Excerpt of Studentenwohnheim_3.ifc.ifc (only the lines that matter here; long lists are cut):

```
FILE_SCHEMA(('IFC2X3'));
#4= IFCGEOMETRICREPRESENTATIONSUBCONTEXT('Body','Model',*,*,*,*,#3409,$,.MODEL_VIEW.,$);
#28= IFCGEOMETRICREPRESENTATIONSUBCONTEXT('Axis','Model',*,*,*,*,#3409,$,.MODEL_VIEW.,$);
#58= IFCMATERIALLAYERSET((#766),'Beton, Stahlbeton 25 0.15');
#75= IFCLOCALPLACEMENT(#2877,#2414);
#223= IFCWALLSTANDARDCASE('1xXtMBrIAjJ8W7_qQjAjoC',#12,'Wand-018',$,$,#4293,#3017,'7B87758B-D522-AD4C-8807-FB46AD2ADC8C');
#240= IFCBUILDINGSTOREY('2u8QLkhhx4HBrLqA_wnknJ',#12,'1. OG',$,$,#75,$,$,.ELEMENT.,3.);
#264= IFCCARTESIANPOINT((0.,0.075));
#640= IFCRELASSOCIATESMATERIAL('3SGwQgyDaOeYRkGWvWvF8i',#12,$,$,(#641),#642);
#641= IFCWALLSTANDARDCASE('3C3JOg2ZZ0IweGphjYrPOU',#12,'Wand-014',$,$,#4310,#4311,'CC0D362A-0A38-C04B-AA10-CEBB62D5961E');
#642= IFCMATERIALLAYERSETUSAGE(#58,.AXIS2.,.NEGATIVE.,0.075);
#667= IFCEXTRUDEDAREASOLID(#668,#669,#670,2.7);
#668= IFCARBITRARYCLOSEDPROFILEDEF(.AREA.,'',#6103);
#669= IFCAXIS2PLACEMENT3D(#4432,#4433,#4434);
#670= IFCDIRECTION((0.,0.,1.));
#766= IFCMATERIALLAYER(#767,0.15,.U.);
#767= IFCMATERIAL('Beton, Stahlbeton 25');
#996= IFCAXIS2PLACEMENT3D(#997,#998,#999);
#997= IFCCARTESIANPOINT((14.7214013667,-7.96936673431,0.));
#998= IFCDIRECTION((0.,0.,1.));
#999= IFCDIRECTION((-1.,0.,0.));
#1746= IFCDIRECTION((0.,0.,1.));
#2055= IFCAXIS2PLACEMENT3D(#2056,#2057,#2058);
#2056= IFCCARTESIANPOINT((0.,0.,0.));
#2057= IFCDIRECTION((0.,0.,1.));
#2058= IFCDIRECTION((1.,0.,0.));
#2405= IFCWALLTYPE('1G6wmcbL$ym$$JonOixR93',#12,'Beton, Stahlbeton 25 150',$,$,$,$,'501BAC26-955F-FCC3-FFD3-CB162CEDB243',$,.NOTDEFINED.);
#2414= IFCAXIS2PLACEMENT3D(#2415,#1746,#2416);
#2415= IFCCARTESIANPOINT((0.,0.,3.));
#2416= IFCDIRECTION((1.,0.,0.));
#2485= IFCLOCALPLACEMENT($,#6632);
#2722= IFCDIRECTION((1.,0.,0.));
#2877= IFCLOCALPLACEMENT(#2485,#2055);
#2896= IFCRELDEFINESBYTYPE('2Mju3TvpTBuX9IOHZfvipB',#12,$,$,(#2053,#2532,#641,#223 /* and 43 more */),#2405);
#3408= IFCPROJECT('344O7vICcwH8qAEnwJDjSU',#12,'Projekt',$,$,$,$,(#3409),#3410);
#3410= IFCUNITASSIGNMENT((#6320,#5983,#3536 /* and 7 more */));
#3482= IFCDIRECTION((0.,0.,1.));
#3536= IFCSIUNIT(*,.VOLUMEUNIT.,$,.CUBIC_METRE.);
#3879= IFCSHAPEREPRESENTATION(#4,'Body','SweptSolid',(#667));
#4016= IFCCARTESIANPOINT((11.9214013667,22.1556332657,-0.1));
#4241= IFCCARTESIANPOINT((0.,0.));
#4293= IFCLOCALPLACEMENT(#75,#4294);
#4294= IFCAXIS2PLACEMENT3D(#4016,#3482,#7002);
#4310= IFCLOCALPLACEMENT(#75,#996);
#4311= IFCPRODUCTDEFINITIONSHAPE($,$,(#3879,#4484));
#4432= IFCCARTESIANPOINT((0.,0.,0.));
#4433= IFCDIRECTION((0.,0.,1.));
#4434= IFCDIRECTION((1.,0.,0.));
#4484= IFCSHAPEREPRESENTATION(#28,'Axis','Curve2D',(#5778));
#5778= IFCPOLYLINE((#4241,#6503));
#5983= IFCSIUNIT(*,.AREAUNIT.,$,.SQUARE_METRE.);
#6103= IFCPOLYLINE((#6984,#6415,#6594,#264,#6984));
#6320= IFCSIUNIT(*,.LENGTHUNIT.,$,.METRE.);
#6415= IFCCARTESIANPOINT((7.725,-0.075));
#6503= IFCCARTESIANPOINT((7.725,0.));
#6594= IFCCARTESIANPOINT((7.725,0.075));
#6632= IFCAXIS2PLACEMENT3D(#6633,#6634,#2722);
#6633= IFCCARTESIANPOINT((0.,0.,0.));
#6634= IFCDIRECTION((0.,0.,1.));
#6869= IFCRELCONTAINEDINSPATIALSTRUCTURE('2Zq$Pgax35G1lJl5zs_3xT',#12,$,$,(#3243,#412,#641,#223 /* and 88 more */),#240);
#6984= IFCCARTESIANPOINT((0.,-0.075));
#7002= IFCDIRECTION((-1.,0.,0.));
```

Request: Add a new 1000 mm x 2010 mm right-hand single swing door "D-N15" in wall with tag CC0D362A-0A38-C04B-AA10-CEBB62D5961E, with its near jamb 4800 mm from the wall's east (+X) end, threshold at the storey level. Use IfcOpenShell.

```python
import numpy as np
import ifcopenshell
import ifcopenshell.api.feature
import ifcopenshell.api.geometry
import ifcopenshell.api.root
import ifcopenshell.api.spatial
import ifcopenshell.api.type
import ifcopenshell.geom
import ifcopenshell.util.element
import ifcopenshell.util.placement
import ifcopenshell.util.representation
import ifcopenshell.util.shape
import ifcopenshell.util.unit

model = ifcopenshell.open("Studentenwohnheim_3.ifc.ifc")
unit_scale = ifcopenshell.util.unit.calculate_unit_scale(model)
settings = ifcopenshell.geom.settings()


def volume(element):
    """Net volume in cubic metres, openings subtracted."""
    shape = ifcopenshell.geom.create_shape(settings, element)
    return ifcopenshell.util.shape.get_volume(shape.geometry)


wall = model.by_id(641)
storey = ifcopenshell.util.element.get_container(wall, ifc_class="IfcBuildingStorey")
context = ifcopenshell.util.representation.get_context(model, "Model", "Body", "MODEL_VIEW")
before = volume(wall)

width, height, from_end, sill = 1, 2.01, 4.8, 0.0  # metres

# The wall runs along its own X axis, and the end named is its -X end.
wall_shape = ifcopenshell.geom.create_shape(settings, wall)
x, y, z = ifcopenshell.util.shape.get_vertices(wall_shape.geometry).T
start = x.min() + from_end
face, thickness = float(y.min()), float(y.max() - y.min())
wall_matrix = ifcopenshell.util.placement.get_local_placement(wall.ObjectPlacement)
level = ifcopenshell.util.placement.get_local_placement(storey.ObjectPlacement)[2, 3]


def in_wall(x, y):
    """Placement at x, y metres in the wall's axes, at sill height."""
    matrix = wall_matrix.copy()
    matrix[:, 3] = wall_matrix @ np.array([x / unit_scale, y / unit_scale, 0.0, 1.0])
    matrix[2, 3] = level + sill / unit_scale
    return matrix


# Opening: a box that overshoots both wall faces by 50 mm.
opening = ifcopenshell.api.root.create_entity(model, ifc_class="IfcOpeningElement")
box = ifcopenshell.api.geometry.add_wall_representation(
    model, context=context, length=width, height=height, thickness=thickness + 0.1
)
ifcopenshell.api.geometry.assign_representation(model, product=opening, representation=box)
ifcopenshell.api.geometry.edit_object_placement(model, product=opening, matrix=in_wall(start, face - 0.05), is_si=False)
ifcopenshell.api.feature.add_feature(model, feature=opening, element=wall)

door = ifcopenshell.api.root.create_entity(model, ifc_class="IfcDoor", name="D-N15")
door.OverallWidth, door.OverallHeight = width / unit_scale, height / unit_scale
body = ifcopenshell.api.geometry.add_door_representation(
    model,
    context=context,
    overall_width=door.OverallWidth,
    overall_height=door.OverallHeight,
    operation_type="SINGLE_SWING_RIGHT",
    lining_properties={"LiningDepth": thickness / unit_scale, "ThresholdDepth": thickness / unit_scale},
)
ifcopenshell.api.geometry.assign_representation(model, product=door, representation=body)
ifcopenshell.api.spatial.assign_container(model, products=[door], relating_structure=storey)
fills = ifcopenshell.api.feature.add_filling(model, opening=opening, element=door)
fills.OwnerHistory = door.OwnerHistory  # required in IFC2X3

# IFC2X3 keeps the operation on the door style.
style = ifcopenshell.api.root.create_entity(model, ifc_class="IfcDoorStyle", name="D-N15")
style.OperationType, style.ConstructionType = "SINGLE_SWING_RIGHT", "NOTDEFINED"
style.ParameterTakesPrecedence = style.Sizeable = False
ifcopenshell.api.type.assign_type(model, related_objects=[door], relating_type=style)

# The lining spans the wall, so the door starts at the wall face.
ifcopenshell.api.geometry.edit_object_placement(model, product=door, matrix=in_wall(start, face), is_si=False)

after = volume(wall)

print(f"wall volume {before:.3f} -> {after:.3f} m3")

model.write("Studentenwohnheim_3.ifc_updated.ifc")
```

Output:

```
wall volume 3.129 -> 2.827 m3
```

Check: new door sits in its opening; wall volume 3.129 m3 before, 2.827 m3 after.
